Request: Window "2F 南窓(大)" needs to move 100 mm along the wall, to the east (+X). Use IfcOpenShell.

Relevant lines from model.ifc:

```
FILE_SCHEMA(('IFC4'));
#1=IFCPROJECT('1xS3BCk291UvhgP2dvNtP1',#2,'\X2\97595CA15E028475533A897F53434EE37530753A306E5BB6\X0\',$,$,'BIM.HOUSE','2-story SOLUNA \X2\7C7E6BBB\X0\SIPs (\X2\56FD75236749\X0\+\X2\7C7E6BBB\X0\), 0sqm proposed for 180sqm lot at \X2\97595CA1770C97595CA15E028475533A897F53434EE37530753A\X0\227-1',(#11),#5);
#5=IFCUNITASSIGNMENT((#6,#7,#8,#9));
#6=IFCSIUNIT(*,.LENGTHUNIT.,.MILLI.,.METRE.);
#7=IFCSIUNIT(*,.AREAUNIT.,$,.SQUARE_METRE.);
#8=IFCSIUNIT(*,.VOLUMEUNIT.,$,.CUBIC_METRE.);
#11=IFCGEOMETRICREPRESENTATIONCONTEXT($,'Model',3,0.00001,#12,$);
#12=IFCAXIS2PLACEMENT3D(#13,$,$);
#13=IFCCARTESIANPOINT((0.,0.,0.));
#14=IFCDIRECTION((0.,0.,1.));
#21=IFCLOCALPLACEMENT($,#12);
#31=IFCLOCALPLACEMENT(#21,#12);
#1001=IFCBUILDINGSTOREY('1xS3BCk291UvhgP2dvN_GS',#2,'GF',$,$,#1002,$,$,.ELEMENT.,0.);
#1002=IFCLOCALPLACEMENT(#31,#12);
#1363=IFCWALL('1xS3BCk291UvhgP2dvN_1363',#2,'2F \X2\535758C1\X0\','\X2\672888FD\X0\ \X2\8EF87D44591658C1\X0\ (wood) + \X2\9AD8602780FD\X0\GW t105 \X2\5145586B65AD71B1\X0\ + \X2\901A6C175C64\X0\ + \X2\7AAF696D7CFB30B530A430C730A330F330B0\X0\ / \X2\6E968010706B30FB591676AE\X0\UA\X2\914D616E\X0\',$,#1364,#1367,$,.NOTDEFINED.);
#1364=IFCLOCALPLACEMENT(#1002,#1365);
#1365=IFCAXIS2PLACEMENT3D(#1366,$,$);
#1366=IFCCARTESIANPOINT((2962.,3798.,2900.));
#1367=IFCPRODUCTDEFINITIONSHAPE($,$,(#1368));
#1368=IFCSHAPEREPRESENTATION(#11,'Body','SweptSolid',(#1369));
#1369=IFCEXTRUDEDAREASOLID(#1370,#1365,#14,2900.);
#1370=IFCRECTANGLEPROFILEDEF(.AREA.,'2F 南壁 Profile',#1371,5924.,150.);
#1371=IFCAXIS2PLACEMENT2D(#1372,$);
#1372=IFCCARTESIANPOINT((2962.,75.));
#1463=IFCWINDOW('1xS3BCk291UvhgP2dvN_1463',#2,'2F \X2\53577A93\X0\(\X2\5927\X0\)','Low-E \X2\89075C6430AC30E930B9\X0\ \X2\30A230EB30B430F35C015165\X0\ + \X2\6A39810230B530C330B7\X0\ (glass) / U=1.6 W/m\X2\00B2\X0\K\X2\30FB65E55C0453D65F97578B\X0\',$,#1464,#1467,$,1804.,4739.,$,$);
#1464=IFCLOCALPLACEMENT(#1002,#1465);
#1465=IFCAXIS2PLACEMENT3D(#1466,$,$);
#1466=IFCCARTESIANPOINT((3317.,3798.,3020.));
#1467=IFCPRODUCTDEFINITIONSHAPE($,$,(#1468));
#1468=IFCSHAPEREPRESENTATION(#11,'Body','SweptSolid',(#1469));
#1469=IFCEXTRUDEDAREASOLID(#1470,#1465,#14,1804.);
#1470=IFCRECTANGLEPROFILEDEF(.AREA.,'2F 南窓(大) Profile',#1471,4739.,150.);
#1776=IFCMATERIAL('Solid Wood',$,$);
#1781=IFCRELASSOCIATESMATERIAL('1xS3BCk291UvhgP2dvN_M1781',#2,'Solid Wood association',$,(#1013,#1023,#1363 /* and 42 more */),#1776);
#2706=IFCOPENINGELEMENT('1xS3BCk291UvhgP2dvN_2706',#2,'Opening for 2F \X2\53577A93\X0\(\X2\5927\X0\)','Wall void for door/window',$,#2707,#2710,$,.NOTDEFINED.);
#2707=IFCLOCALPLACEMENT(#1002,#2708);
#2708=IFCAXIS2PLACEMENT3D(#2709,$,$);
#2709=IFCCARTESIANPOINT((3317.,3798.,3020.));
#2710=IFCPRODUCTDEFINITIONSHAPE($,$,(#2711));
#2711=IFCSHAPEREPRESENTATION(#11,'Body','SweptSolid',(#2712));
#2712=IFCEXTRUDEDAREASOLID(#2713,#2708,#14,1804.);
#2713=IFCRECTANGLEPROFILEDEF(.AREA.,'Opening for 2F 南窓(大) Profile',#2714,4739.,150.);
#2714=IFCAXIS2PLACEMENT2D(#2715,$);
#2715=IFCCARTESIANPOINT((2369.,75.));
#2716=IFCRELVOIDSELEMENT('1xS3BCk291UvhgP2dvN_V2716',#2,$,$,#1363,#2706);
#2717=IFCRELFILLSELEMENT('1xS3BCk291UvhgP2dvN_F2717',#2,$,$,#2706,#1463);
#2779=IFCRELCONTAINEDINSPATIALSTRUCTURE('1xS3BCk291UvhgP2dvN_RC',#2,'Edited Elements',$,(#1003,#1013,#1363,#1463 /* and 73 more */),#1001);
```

```python
import ifcopenshell
import ifcopenshell.api.geometry
import ifcopenshell.util.placement

model = ifcopenshell.open("model.ifc")

window = model.by_guid("1xS3BCk291UvhgP2dvN_1463")
opening = window.FillsVoids[0].RelatingOpeningElement
wall = opening.VoidsElements[0].RelatingBuildingElement

wall_matrix = ifcopenshell.util.placement.get_local_placement(wall.ObjectPlacement)
shift = wall_matrix[:3, 0] * 100.0
before = ifcopenshell.util.placement.get_local_placement(window.ObjectPlacement)[:3, 3].copy()

# The window is not placed relative to its opening, so move both.
for product in (opening, window):
    matrix = ifcopenshell.util.placement.get_local_placement(product.ObjectPlacement)
    matrix[:3, 3] += shift
    ifcopenshell.api.geometry.edit_object_placement(model, product=product, matrix=matrix, is_si=False)

after = ifcopenshell.util.placement.get_local_placement(window.ObjectPlacement)[:3, 3]
print("window moved by", (after - before).round(3) + 0.0)

model.write("model_rev.ifc")
```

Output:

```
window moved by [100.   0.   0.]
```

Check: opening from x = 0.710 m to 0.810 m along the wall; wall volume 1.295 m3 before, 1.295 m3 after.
